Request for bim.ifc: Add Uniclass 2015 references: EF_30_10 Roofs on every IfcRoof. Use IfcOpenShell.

First a look at what the model holds.

```python
import ifcopenshell

model = ifcopenshell.open("bim.ifc")
print(model.schema)
print("classifications:", [c.Name for c in model.by_type("IfcClassification")])
for ifc_class in ("IfcDoor", "IfcRoof", "IfcStair", "IfcWall", "IfcWindow"):
    print(ifc_class, len(model.by_type(ifc_class)))
```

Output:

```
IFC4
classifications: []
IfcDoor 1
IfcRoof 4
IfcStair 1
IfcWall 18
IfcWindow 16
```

```python
import ifcopenshell
import ifcopenshell.api.classification

model = ifcopenshell.open("bim.ifc")

system = ifcopenshell.api.classification.add_classification(model, classification="Uniclass 2015")

codes = {
    "IfcRoof": ("EF_30_10", "Roofs"),
}
for ifc_class, (code, name) in codes.items():
    products = model.by_type(ifc_class)
    ifcopenshell.api.classification.add_reference(
        model, products=products, classification=system, identification=code, name=name
    )
    print(code, len(products))

model.write("bim_edited.ifc")
```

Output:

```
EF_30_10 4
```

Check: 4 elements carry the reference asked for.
